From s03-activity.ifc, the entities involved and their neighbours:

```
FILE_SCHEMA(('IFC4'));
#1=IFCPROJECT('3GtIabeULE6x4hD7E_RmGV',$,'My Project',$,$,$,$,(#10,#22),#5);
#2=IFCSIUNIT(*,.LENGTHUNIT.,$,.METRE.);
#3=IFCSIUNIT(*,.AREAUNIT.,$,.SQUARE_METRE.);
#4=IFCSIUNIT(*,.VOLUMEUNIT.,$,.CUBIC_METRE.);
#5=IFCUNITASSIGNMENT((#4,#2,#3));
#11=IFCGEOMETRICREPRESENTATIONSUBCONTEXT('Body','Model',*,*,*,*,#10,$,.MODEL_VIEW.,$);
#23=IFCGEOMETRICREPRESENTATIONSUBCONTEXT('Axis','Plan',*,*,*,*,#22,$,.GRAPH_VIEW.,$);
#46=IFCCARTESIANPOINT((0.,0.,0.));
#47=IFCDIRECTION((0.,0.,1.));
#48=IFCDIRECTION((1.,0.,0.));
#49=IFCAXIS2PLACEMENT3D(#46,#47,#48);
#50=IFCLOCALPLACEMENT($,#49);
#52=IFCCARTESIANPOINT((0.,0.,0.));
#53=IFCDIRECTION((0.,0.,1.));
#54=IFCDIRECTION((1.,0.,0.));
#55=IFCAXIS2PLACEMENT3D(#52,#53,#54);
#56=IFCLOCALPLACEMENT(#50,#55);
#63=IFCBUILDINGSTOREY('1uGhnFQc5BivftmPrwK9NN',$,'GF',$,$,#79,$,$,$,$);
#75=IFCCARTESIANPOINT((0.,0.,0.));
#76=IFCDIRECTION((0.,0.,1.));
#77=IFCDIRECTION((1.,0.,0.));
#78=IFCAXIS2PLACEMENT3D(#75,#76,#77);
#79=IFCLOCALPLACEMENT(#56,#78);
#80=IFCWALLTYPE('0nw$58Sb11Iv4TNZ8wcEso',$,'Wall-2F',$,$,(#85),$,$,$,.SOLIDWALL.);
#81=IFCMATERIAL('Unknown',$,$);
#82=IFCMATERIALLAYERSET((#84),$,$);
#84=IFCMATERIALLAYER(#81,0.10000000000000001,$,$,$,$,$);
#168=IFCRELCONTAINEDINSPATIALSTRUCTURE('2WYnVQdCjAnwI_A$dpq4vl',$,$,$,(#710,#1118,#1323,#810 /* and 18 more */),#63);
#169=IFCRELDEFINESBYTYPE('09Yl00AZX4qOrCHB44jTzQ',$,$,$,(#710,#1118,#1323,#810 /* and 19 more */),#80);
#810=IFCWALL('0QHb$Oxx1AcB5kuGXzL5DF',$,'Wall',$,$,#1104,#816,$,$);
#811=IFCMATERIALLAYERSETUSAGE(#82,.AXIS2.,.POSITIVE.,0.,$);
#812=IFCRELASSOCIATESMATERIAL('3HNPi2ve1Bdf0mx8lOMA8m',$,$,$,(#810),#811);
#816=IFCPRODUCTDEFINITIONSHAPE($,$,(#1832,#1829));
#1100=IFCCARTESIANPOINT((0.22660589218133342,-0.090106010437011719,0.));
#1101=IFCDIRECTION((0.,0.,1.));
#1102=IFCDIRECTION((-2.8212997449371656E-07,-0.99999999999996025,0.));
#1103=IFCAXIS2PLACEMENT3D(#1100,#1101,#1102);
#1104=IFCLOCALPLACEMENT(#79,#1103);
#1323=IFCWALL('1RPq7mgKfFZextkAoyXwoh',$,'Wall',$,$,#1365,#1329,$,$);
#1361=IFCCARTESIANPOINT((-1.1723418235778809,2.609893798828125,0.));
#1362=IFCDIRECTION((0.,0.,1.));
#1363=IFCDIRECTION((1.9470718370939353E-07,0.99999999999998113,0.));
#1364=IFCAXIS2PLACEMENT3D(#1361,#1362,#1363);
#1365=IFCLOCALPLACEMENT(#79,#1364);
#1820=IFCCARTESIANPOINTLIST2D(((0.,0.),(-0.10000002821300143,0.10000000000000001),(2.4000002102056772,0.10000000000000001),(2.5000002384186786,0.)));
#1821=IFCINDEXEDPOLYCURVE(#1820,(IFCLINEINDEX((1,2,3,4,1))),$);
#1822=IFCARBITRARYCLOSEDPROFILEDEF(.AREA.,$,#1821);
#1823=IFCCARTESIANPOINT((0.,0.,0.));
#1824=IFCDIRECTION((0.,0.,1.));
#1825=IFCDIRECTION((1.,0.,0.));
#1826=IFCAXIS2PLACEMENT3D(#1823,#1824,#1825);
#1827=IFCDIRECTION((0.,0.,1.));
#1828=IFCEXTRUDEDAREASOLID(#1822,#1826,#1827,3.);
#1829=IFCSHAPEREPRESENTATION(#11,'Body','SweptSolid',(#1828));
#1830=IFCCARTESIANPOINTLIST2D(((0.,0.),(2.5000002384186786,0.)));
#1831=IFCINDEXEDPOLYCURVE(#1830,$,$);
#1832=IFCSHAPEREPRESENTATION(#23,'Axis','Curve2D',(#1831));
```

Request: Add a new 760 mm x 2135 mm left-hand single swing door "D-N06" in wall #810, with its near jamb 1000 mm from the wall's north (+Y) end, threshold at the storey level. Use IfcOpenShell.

```python
import numpy as np
import ifcopenshell
import ifcopenshell.api.feature
import ifcopenshell.api.geometry
import ifcopenshell.api.root
import ifcopenshell.api.spatial
import ifcopenshell.geom
import ifcopenshell.util.element
import ifcopenshell.util.placement
import ifcopenshell.util.representation
import ifcopenshell.util.shape
import ifcopenshell.util.unit

model = ifcopenshell.open("s03-activity.ifc")
unit_scale = ifcopenshell.util.unit.calculate_unit_scale(model)
settings = ifcopenshell.geom.settings()


def volume(element):
    """Net volume in cubic metres, openings subtracted."""
    shape = ifcopenshell.geom.create_shape(settings, element)
    return ifcopenshell.util.shape.get_volume(shape.geometry)


wall = model.by_guid("0QHb$Oxx1AcB5kuGXzL5DF")
storey = ifcopenshell.util.element.get_container(wall, ifc_class="IfcBuildingStorey")
context = ifcopenshell.util.representation.get_context(model, "Model", "Body", "MODEL_VIEW")
before = volume(wall)

width, height, from_end, sill = 0.76, 2.135, 1, 0.0  # metres

# The wall runs along its own X axis, and the end named is its -X end.
wall_shape = ifcopenshell.geom.create_shape(settings, wall)
x, y, z = ifcopenshell.util.shape.get_vertices(wall_shape.geometry).T
start = x.min() + from_end
face, thickness = float(y.min()), float(y.max() - y.min())
wall_matrix = ifcopenshell.util.placement.get_local_placement(wall.ObjectPlacement)
level = ifcopenshell.util.placement.get_local_placement(storey.ObjectPlacement)[2, 3]


def in_wall(x, y):
    """Placement at x, y metres in the wall's axes, at sill height."""
    matrix = wall_matrix.copy()
    matrix[:, 3] = wall_matrix @ np.array([x / unit_scale, y / unit_scale, 0.0, 1.0])
    matrix[2, 3] = level + sill / unit_scale
    return matrix


# Opening: a box that overshoots both wall faces by 50 mm.
opening = ifcopenshell.api.root.create_entity(model, ifc_class="IfcOpeningElement", predefined_type="OPENING")
box = ifcopenshell.api.geometry.add_wall_representation(
    model, context=context, length=width, height=height, thickness=thickness + 0.1
)
ifcopenshell.api.geometry.assign_representation(model, product=opening, representation=box)
ifcopenshell.api.geometry.edit_object_placement(model, product=opening, matrix=in_wall(start, face - 0.05), is_si=False)
ifcopenshell.api.feature.add_feature(model, feature=opening, element=wall)

door = ifcopenshell.api.root.create_entity(model, ifc_class="IfcDoor", name="D-N06", predefined_type="DOOR")
door.OverallWidth, door.OverallHeight = width / unit_scale, height / unit_scale
door.OperationType = "SINGLE_SWING_LEFT"
body = ifcopenshell.api.geometry.add_door_representation(
    model,
    context=context,
    overall_width=door.OverallWidth,
    overall_height=door.OverallHeight,
    operation_type="SINGLE_SWING_LEFT",
    lining_properties={"LiningDepth": thickness / unit_scale, "ThresholdDepth": thickness / unit_scale},
)
ifcopenshell.api.geometry.assign_representation(model, product=door, representation=body)
ifcopenshell.api.spatial.assign_container(model, products=[door], relating_structure=storey)
ifcopenshell.api.feature.add_filling(model, opening=opening, element=door)

# The lining spans the wall, so the door starts at the wall face.
ifcopenshell.api.geometry.edit_object_placement(model, product=door, matrix=in_wall(start, face), is_si=False)

after = volume(wall)

print(f"wall volume {before:.3f} -> {after:.3f} m3")

model.write("s03-activity_edited.ifc")
```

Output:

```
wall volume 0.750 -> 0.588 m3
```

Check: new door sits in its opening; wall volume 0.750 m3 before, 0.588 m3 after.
